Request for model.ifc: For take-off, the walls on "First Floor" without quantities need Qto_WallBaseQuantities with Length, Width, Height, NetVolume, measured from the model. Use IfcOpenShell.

First a look at what the model holds.

```python
import ifcopenshell
import ifcopenshell.util.element
import ifcopenshell.util.unit

model = ifcopenshell.open("model.ifc")
print(model.schema)
for unit_type in ("LENGTHUNIT", "AREAUNIT", "VOLUMEUNIT"):
    print(unit_type, ifcopenshell.util.unit.calculate_unit_scale(model, unit_type))
storey = next(s for s in model.by_type("IfcBuildingStorey") if s.Name == "First Floor")
walls = [e for e in ifcopenshell.util.element.get_decomposition(storey) if e.is_a("IfcWall")]
for e in sorted(walls, key=lambda e: e.id()):
    print(e.id(), e.is_a(), e.Name, list(ifcopenshell.util.element.get_psets(e, qtos_only=True)), sep=" | ")
```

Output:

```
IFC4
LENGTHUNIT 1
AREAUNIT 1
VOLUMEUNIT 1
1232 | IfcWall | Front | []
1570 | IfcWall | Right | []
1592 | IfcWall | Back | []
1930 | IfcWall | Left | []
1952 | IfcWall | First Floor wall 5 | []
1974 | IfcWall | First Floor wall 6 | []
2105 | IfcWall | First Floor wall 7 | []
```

```python
import ifcopenshell
import ifcopenshell.api.pset
import ifcopenshell.geom
import ifcopenshell.util.element
import ifcopenshell.util.shape
import ifcopenshell.util.unit

model = ifcopenshell.open("model.ifc")
unit_scale = ifcopenshell.util.unit.calculate_unit_scale(model)
volume_scale = ifcopenshell.util.unit.calculate_unit_scale(model, "VOLUMEUNIT")
settings = ifcopenshell.geom.settings()

storey = next(s for s in model.by_type("IfcBuildingStorey") if s.Name == "First Floor")
walls = [e for e in ifcopenshell.util.element.get_decomposition(storey) if e.is_a("IfcWall")]

for e in sorted(walls, key=lambda e: e.id()):
    if ifcopenshell.util.element.get_psets(e, qtos_only=True, should_inherit=False):
        continue
    # Geometry comes back in metres, in the element's own axes.
    shape = ifcopenshell.geom.create_shape(settings, e)
    values = {
        "Length": ifcopenshell.util.shape.get_x(shape.geometry) / unit_scale,
        "Width": ifcopenshell.util.shape.get_y(shape.geometry) / unit_scale,
        "Height": ifcopenshell.util.shape.get_z(shape.geometry) / unit_scale,
        "NetVolume": ifcopenshell.util.shape.get_volume(shape.geometry) / volume_scale,
    }
    qto = ifcopenshell.api.pset.add_qto(model, product=e, name="Qto_WallBaseQuantities")
    ifcopenshell.api.pset.edit_qto(model, qto=qto, properties=values)
    print(e.id(), {k: round(v, 3) for k, v in values.items()})

model.write("model-out.ifc")
```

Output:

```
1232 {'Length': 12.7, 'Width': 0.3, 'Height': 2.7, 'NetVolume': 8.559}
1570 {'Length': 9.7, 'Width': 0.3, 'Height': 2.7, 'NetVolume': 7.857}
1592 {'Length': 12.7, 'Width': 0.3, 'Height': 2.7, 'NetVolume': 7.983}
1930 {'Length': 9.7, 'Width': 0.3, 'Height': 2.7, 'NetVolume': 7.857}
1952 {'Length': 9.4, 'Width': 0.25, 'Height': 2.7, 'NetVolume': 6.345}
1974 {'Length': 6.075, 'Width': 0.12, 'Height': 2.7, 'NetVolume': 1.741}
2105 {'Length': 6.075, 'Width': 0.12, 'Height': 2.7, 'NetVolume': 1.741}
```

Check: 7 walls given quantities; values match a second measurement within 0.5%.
